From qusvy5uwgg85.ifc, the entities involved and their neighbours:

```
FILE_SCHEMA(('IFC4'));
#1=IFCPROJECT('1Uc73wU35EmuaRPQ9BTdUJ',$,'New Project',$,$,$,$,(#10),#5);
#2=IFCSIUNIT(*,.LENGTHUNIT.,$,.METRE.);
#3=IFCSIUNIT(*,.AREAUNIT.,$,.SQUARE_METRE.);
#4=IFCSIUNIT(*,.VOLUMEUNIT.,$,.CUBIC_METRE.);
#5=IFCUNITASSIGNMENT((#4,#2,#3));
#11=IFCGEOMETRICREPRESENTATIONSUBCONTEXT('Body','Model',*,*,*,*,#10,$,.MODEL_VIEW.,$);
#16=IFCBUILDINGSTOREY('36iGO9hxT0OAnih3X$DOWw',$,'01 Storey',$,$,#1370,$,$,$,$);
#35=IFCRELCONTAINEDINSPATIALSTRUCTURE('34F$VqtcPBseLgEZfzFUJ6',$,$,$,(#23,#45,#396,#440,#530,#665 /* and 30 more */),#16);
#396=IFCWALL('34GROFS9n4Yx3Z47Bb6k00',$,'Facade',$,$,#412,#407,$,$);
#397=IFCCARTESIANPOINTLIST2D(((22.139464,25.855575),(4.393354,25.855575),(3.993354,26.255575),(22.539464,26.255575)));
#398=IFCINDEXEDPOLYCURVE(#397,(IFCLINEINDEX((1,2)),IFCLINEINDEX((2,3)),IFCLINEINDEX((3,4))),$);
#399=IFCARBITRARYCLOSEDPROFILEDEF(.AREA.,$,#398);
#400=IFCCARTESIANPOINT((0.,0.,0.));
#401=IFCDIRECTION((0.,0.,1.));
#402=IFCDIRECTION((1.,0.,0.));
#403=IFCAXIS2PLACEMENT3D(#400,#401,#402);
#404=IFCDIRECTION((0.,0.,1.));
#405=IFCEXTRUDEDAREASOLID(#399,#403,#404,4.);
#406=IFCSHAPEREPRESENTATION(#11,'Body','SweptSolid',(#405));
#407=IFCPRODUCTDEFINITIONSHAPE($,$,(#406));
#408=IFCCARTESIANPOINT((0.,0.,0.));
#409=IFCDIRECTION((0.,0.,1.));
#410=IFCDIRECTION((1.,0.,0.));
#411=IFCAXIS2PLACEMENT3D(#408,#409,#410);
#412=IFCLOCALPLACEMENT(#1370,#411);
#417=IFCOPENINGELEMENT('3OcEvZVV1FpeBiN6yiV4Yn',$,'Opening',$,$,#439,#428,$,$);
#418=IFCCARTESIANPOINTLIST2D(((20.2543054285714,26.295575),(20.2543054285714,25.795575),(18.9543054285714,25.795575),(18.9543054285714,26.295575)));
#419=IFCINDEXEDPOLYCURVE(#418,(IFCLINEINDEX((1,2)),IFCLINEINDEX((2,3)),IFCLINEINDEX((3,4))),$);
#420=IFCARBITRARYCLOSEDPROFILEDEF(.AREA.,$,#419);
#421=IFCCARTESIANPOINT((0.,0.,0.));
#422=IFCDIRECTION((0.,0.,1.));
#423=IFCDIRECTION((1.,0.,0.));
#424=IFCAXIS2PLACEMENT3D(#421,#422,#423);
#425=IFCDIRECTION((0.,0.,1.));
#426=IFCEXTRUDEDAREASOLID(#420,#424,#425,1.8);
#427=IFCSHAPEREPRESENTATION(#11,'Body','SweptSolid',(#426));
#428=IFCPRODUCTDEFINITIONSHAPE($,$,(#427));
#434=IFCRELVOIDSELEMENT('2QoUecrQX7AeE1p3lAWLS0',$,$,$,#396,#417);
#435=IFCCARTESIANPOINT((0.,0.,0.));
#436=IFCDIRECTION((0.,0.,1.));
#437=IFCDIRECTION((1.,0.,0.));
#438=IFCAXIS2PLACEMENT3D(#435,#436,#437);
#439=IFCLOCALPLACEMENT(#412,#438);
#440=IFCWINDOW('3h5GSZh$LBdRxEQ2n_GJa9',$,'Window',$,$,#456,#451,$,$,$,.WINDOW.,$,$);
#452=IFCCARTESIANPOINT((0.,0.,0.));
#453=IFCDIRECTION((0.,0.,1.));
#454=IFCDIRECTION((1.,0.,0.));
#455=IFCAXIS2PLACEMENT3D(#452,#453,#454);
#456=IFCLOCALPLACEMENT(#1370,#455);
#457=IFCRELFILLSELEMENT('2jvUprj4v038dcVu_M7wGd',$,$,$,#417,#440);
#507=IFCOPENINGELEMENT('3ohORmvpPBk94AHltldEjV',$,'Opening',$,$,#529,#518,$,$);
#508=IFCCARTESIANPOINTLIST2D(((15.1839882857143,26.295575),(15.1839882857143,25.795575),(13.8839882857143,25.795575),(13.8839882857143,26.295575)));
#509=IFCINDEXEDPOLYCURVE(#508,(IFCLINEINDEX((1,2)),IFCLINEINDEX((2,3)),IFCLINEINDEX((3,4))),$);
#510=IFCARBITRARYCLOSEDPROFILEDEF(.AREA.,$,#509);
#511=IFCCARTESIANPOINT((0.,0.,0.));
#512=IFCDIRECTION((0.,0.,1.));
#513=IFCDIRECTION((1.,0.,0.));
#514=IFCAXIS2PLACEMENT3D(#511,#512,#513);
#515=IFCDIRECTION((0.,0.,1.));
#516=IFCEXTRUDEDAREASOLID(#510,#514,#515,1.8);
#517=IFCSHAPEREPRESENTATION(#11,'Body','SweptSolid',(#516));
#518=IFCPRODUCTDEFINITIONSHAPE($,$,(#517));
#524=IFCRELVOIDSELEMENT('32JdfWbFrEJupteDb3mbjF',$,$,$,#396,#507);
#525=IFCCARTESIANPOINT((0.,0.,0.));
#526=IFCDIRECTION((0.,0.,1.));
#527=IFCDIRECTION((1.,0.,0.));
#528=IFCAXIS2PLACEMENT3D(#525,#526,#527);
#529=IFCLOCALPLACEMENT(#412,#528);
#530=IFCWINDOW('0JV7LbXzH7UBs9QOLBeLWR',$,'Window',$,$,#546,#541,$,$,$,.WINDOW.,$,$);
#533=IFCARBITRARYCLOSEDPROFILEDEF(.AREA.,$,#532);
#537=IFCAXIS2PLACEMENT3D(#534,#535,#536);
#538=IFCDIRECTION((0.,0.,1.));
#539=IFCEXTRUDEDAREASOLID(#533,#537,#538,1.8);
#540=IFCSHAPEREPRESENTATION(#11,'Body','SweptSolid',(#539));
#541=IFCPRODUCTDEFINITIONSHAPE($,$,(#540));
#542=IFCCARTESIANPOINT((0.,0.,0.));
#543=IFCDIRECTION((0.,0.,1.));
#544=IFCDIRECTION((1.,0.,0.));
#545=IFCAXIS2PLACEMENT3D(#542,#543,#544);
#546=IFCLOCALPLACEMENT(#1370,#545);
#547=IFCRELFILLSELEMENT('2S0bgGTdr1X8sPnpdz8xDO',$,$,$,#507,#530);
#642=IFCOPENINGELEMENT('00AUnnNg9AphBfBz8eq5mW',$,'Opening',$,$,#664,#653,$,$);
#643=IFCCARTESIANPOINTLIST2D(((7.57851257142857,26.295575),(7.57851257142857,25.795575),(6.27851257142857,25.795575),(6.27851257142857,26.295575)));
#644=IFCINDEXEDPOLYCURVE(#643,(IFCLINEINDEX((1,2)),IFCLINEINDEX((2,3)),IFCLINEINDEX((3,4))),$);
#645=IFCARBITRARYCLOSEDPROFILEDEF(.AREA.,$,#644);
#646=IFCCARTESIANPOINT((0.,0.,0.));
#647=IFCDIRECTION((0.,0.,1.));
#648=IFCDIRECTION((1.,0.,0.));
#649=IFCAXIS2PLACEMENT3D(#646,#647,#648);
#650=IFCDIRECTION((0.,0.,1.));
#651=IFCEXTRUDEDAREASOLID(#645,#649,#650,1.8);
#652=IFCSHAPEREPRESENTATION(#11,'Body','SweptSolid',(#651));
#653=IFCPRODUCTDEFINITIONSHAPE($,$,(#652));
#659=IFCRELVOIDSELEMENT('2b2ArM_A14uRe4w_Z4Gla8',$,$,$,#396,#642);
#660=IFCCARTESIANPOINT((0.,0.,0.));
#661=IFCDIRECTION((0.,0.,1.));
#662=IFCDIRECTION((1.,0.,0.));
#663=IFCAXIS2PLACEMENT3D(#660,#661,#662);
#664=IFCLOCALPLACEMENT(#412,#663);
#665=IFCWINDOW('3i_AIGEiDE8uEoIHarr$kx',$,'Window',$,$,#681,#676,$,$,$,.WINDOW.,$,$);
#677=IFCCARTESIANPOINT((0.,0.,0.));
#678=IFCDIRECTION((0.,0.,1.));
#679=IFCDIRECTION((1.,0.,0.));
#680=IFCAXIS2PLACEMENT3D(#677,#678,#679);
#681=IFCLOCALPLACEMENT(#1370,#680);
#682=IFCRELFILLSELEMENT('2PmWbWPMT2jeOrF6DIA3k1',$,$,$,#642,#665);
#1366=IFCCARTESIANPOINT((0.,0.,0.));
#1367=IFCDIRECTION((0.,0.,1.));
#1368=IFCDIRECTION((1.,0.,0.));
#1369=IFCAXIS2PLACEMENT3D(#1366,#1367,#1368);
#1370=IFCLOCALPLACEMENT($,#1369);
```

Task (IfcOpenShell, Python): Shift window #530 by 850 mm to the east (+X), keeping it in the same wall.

```python
import ifcopenshell
import ifcopenshell.api.geometry
import ifcopenshell.util.placement
import ifcopenshell.util.unit

model = ifcopenshell.open("qusvy5uwgg85.ifc")
unit_scale = ifcopenshell.util.unit.calculate_unit_scale(model)

window = model.by_guid("0JV7LbXzH7UBs9QOLBeLWR")
opening = window.FillsVoids[0].RelatingOpeningElement
wall = opening.VoidsElements[0].RelatingBuildingElement

wall_matrix = ifcopenshell.util.placement.get_local_placement(wall.ObjectPlacement)
shift = wall_matrix[:3, 0] * 0.85 / unit_scale
before = ifcopenshell.util.placement.get_local_placement(window.ObjectPlacement)[:3, 3].copy()

# The window is not placed relative to its opening, so move both.
for product in (opening, window):
    matrix = ifcopenshell.util.placement.get_local_placement(product.ObjectPlacement)
    matrix[:3, 3] += shift
    ifcopenshell.api.geometry.edit_object_placement(model, product=product, matrix=matrix, is_si=False)

after = ifcopenshell.util.placement.get_local_placement(window.ObjectPlacement)[:3, 3]
print("window moved by", (after - before).round(3) + 0.0)

model.write("qusvy5uwgg85_updated.ifc")
```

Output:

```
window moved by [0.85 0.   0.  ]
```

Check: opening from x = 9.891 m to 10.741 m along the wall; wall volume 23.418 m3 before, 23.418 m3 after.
